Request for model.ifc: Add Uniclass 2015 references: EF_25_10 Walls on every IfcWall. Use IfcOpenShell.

First a look at what the model holds.

```python
import ifcopenshell

model = ifcopenshell.open("model.ifc")
print(model.schema)
print("classifications:", [c.Name for c in model.by_type("IfcClassification")])
for ifc_class in ("IfcDoor", "IfcRoof", "IfcStair", "IfcWall", "IfcWindow"):
    print(ifc_class, len(model.by_type(ifc_class)))
```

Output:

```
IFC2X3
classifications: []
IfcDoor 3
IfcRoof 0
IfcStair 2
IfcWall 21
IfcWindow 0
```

```python
import ifcopenshell
import ifcopenshell.api.classification

model = ifcopenshell.open("model.ifc")

# IFC2X3 requires Source and Edition and has no link from the project to the system.
system = model.create_entity("IfcClassification", Source="NBS", Edition="2015", Name="Uniclass 2015")

codes = {
    "IfcWall": ("EF_25_10", "Walls"),
}
for ifc_class, (code, name) in codes.items():
    products = model.by_type(ifc_class)
    ifcopenshell.api.classification.add_reference(
        model, products=products, classification=system, identification=code, name=name
    )
    print(code, len(products))

model.write("model-out.ifc")
```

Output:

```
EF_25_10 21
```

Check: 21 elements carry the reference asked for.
